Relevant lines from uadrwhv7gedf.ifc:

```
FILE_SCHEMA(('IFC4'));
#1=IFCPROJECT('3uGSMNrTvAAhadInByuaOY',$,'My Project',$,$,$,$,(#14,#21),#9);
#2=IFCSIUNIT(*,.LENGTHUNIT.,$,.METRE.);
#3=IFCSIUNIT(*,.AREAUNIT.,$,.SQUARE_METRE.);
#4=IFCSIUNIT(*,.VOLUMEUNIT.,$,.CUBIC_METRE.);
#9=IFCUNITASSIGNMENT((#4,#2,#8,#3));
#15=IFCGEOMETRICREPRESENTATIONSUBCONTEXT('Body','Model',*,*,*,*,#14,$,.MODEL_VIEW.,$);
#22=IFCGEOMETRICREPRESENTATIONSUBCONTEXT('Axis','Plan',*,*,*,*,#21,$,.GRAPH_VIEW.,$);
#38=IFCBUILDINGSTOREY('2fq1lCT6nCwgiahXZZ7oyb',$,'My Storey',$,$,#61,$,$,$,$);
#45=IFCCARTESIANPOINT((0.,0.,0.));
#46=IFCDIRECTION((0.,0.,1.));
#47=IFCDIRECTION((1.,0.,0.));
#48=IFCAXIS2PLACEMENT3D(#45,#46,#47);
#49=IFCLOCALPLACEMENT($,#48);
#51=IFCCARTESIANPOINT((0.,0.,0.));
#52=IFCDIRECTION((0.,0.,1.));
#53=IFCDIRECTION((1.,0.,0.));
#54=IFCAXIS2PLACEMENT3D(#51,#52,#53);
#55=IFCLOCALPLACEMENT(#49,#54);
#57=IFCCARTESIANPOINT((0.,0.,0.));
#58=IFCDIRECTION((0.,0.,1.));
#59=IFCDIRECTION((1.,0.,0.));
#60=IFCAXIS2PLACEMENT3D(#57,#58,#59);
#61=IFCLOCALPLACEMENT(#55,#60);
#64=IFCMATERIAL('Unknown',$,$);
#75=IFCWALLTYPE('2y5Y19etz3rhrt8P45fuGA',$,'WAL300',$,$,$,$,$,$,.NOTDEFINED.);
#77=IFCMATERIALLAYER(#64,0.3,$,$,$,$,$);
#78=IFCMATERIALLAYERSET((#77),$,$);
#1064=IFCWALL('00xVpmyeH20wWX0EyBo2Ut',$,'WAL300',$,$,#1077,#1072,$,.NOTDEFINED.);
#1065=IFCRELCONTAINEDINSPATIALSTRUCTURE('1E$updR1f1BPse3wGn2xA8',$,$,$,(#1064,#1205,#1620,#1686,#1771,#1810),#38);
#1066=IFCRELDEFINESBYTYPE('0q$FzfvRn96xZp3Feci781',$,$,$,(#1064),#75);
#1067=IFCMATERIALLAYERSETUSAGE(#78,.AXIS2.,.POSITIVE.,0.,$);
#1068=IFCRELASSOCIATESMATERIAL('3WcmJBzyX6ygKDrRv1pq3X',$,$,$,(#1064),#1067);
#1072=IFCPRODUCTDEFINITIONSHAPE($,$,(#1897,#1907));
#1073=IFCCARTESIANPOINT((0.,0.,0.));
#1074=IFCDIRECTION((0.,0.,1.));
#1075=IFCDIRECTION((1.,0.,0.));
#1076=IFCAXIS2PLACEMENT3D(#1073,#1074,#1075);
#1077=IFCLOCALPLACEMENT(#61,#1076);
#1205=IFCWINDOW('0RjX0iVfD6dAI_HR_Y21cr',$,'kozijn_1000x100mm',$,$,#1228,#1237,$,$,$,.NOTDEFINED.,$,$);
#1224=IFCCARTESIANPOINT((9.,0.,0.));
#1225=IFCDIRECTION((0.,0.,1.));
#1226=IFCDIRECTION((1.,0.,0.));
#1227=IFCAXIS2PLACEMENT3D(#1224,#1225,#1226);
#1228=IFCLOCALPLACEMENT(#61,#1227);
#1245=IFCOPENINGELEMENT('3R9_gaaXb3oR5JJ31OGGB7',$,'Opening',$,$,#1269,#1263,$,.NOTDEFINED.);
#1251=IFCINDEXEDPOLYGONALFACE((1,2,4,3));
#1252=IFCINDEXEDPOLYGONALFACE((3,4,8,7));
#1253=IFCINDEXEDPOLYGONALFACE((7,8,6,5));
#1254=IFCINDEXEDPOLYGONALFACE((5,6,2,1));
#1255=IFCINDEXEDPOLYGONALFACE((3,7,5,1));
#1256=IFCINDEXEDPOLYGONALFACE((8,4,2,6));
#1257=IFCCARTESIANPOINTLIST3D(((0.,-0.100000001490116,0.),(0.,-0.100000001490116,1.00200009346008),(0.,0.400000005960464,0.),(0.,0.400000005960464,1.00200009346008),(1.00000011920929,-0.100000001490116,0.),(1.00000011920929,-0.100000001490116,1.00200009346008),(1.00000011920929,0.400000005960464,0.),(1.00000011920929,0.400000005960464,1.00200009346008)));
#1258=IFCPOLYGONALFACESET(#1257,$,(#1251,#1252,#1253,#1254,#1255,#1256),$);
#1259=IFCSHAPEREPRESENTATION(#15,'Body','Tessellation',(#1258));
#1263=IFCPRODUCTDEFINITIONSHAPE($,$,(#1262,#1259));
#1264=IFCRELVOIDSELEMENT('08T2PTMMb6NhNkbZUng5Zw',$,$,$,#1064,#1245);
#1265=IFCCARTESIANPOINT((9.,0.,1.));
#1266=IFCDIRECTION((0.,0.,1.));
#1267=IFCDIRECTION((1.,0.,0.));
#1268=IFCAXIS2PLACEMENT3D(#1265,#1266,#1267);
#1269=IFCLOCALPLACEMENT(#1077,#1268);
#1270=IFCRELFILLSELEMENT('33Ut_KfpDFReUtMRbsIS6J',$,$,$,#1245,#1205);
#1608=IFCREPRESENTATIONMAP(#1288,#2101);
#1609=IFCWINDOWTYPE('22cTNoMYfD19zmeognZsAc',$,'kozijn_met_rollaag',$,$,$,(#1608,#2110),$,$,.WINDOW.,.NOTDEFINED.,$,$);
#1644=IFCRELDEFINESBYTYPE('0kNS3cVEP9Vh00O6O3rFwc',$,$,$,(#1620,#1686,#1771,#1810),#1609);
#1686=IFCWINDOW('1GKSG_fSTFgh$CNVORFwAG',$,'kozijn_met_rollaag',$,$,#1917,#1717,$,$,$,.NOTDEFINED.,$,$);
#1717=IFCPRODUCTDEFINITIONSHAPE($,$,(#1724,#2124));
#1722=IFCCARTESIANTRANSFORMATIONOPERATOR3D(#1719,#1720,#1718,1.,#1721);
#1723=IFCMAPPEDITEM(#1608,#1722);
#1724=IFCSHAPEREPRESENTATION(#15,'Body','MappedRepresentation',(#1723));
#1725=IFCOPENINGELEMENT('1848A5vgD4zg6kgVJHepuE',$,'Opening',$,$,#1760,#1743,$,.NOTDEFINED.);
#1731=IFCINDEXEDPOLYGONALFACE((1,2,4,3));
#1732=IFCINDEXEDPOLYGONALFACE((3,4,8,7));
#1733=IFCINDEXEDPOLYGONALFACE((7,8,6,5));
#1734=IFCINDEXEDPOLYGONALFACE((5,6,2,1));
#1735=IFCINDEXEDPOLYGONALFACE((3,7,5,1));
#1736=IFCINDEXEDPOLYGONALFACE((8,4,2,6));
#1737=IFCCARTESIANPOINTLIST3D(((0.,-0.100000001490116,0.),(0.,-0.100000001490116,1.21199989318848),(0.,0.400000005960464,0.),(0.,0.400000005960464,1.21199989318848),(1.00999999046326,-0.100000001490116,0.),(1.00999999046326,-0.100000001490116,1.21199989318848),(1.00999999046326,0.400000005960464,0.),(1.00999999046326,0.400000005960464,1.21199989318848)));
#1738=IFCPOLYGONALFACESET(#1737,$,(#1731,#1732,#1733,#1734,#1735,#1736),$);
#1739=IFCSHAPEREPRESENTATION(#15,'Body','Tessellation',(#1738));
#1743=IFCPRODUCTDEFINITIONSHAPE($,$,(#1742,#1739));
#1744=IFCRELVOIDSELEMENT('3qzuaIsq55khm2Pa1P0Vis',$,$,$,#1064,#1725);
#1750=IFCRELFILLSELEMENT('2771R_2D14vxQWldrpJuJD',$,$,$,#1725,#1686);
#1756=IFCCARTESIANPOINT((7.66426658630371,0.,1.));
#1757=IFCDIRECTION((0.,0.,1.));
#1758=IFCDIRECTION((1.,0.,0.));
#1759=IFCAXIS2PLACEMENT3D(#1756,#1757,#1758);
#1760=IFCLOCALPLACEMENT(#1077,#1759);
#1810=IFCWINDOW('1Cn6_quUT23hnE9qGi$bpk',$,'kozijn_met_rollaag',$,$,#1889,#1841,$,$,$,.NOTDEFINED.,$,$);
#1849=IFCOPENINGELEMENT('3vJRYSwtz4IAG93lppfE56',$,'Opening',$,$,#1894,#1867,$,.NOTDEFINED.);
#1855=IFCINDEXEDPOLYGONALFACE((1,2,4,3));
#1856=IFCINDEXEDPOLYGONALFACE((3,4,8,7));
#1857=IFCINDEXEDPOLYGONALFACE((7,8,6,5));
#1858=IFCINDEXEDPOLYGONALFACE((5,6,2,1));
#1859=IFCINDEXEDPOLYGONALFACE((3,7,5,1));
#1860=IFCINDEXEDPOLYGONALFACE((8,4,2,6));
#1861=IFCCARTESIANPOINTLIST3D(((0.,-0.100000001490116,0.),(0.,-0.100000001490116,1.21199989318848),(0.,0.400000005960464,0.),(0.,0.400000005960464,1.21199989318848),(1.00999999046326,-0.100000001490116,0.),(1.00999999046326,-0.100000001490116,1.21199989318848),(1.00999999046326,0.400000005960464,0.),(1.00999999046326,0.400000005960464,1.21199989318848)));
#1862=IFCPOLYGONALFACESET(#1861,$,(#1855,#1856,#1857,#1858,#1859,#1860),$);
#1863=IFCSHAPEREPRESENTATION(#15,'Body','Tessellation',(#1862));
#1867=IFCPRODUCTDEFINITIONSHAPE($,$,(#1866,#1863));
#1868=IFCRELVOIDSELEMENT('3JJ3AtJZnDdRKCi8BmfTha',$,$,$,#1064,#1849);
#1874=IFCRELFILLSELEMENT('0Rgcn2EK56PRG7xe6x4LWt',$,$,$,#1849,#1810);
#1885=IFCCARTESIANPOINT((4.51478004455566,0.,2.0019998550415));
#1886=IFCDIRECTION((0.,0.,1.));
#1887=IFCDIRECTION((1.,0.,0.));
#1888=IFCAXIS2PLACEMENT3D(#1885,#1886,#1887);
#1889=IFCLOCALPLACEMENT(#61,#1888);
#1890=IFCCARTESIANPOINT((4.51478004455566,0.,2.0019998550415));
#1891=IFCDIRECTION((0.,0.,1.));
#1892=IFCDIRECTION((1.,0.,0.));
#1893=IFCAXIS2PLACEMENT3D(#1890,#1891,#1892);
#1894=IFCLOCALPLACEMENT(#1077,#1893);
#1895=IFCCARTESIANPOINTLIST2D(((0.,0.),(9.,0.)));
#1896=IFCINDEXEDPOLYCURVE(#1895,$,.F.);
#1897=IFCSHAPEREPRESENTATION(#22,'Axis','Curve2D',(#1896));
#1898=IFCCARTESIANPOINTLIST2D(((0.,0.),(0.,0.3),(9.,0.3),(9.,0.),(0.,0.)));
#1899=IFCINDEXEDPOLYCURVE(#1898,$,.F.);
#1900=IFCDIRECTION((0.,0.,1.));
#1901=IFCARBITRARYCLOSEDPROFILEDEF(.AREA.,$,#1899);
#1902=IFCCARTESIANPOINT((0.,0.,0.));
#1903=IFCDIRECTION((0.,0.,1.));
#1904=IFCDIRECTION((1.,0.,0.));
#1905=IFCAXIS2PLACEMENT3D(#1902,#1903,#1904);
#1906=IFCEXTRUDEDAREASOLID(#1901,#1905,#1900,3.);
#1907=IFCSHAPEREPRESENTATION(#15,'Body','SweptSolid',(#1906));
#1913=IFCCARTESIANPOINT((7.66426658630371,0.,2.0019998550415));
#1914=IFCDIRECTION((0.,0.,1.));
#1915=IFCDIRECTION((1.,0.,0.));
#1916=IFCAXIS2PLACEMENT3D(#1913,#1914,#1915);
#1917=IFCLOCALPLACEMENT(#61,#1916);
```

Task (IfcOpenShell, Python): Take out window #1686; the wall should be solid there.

```python
import ifcopenshell
import ifcopenshell.api.feature
import ifcopenshell.api.root
import ifcopenshell.geom
import ifcopenshell.util.shape

model = ifcopenshell.open("uadrwhv7gedf.ifc")
settings = ifcopenshell.geom.settings()


def volume(element):
    """Net volume in cubic metres, openings subtracted."""
    shape = ifcopenshell.geom.create_shape(settings, element)
    return ifcopenshell.util.shape.get_volume(shape.geometry)


window = model.by_id(1686)
opening = window.FillsVoids[0].RelatingOpeningElement
wall = opening.VoidsElements[0].RelatingBuildingElement
before = volume(wall)

ifcopenshell.api.root.remove_product(model, product=window)
ifcopenshell.api.feature.remove_feature(model, feature=opening)

after = volume(wall)

print(f"wall volume {before:.3f} -> {after:.3f} m3")

model.write("uadrwhv7gedf_rev.ifc")
```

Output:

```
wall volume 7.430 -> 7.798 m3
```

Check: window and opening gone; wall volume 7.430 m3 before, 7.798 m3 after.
